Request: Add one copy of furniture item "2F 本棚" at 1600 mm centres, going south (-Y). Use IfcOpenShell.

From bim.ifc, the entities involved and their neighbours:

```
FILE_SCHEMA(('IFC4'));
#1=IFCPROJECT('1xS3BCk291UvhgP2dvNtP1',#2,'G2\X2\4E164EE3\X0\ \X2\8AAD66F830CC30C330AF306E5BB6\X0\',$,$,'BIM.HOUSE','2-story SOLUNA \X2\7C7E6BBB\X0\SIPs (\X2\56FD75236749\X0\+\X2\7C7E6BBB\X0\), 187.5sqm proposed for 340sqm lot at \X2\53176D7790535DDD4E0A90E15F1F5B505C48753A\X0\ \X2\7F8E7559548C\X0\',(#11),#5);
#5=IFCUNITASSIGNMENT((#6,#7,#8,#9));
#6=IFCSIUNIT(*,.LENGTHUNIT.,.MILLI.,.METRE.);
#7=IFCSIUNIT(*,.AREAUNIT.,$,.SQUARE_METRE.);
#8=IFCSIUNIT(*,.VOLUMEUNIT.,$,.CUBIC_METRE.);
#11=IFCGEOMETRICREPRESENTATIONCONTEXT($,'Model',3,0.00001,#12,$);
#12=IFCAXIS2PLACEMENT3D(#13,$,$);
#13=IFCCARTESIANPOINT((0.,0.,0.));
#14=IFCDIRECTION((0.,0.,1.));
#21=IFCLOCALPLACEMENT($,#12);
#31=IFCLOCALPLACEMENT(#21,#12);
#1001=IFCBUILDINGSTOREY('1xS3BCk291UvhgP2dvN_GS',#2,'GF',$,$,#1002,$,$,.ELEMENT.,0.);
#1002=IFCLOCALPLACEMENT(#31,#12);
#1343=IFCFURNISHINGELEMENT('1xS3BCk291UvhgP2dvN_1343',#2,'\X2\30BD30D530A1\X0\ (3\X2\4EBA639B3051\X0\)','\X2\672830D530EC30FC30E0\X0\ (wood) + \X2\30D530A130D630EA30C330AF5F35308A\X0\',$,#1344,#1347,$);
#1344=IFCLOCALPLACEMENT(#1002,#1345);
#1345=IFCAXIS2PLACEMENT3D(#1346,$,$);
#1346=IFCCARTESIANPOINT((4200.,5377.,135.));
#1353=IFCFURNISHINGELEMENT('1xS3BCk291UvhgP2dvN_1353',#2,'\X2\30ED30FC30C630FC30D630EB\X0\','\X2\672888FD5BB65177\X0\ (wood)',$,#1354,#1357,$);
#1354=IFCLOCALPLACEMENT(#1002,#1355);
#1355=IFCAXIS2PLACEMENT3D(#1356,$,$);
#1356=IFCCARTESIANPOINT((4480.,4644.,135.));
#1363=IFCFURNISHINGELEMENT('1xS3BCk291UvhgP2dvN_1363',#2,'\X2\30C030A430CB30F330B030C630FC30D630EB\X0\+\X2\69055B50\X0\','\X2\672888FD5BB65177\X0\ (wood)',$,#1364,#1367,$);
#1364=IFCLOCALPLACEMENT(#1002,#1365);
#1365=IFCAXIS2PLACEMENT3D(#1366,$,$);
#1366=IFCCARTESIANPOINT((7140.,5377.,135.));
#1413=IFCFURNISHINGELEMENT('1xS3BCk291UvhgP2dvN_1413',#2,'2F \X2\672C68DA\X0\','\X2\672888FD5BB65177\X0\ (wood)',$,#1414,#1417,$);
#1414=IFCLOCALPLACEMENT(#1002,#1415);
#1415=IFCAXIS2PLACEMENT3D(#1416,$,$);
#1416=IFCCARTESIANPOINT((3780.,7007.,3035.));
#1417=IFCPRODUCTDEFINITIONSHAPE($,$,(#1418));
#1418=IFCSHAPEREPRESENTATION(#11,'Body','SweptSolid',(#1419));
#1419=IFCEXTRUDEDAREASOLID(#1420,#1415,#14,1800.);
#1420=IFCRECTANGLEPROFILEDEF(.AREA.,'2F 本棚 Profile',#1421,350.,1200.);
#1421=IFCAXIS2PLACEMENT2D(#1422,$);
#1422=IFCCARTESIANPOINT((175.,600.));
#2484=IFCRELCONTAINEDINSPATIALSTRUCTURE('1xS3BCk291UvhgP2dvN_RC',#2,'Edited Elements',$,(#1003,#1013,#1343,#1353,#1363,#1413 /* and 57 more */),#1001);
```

```python
import numpy as np
import ifcopenshell
import ifcopenshell.api.geometry
import ifcopenshell.api.root
import ifcopenshell.util.element
import ifcopenshell.util.placement

model = ifcopenshell.open("bim.ifc")


def reuse_history(source, copy):
    """copy_class also copies each property set's owner history, people and application; keep the originals."""
    for rel in copy.IsDefinedBy:
        if rel.is_a("IfcRelDefinesByProperties") and (history := rel.RelatingPropertyDefinition.OwnerHistory):
            rel.RelatingPropertyDefinition.OwnerHistory = source.OwnerHistory
            ifcopenshell.util.element.remove_deep2(model, history)


source = model.by_guid("1xS3BCk291UvhgP2dvN_1413")
base = ifcopenshell.util.placement.get_local_placement(source.ObjectPlacement)
step = np.array([0.0, -1.0, 0.0]) * 1600.0

for i in range(1, 2):
    copy = ifcopenshell.api.root.copy_class(model, product=source)
    copy.Representation = ifcopenshell.util.element.copy_deep(
        model, source.Representation, exclude=["IfcGeometricRepresentationContext", "IfcRepresentationMap"]
    )
    reuse_history(source, copy)
    matrix = base.copy()
    matrix[:3, 3] += i * step
    print("added at", matrix[:3, 3].round(3) + 0.0)
    ifcopenshell.api.geometry.edit_object_placement(model, product=copy, matrix=matrix, is_si=False)

model.write("bim_v2.ifc")
```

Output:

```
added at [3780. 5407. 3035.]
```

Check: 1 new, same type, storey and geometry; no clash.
